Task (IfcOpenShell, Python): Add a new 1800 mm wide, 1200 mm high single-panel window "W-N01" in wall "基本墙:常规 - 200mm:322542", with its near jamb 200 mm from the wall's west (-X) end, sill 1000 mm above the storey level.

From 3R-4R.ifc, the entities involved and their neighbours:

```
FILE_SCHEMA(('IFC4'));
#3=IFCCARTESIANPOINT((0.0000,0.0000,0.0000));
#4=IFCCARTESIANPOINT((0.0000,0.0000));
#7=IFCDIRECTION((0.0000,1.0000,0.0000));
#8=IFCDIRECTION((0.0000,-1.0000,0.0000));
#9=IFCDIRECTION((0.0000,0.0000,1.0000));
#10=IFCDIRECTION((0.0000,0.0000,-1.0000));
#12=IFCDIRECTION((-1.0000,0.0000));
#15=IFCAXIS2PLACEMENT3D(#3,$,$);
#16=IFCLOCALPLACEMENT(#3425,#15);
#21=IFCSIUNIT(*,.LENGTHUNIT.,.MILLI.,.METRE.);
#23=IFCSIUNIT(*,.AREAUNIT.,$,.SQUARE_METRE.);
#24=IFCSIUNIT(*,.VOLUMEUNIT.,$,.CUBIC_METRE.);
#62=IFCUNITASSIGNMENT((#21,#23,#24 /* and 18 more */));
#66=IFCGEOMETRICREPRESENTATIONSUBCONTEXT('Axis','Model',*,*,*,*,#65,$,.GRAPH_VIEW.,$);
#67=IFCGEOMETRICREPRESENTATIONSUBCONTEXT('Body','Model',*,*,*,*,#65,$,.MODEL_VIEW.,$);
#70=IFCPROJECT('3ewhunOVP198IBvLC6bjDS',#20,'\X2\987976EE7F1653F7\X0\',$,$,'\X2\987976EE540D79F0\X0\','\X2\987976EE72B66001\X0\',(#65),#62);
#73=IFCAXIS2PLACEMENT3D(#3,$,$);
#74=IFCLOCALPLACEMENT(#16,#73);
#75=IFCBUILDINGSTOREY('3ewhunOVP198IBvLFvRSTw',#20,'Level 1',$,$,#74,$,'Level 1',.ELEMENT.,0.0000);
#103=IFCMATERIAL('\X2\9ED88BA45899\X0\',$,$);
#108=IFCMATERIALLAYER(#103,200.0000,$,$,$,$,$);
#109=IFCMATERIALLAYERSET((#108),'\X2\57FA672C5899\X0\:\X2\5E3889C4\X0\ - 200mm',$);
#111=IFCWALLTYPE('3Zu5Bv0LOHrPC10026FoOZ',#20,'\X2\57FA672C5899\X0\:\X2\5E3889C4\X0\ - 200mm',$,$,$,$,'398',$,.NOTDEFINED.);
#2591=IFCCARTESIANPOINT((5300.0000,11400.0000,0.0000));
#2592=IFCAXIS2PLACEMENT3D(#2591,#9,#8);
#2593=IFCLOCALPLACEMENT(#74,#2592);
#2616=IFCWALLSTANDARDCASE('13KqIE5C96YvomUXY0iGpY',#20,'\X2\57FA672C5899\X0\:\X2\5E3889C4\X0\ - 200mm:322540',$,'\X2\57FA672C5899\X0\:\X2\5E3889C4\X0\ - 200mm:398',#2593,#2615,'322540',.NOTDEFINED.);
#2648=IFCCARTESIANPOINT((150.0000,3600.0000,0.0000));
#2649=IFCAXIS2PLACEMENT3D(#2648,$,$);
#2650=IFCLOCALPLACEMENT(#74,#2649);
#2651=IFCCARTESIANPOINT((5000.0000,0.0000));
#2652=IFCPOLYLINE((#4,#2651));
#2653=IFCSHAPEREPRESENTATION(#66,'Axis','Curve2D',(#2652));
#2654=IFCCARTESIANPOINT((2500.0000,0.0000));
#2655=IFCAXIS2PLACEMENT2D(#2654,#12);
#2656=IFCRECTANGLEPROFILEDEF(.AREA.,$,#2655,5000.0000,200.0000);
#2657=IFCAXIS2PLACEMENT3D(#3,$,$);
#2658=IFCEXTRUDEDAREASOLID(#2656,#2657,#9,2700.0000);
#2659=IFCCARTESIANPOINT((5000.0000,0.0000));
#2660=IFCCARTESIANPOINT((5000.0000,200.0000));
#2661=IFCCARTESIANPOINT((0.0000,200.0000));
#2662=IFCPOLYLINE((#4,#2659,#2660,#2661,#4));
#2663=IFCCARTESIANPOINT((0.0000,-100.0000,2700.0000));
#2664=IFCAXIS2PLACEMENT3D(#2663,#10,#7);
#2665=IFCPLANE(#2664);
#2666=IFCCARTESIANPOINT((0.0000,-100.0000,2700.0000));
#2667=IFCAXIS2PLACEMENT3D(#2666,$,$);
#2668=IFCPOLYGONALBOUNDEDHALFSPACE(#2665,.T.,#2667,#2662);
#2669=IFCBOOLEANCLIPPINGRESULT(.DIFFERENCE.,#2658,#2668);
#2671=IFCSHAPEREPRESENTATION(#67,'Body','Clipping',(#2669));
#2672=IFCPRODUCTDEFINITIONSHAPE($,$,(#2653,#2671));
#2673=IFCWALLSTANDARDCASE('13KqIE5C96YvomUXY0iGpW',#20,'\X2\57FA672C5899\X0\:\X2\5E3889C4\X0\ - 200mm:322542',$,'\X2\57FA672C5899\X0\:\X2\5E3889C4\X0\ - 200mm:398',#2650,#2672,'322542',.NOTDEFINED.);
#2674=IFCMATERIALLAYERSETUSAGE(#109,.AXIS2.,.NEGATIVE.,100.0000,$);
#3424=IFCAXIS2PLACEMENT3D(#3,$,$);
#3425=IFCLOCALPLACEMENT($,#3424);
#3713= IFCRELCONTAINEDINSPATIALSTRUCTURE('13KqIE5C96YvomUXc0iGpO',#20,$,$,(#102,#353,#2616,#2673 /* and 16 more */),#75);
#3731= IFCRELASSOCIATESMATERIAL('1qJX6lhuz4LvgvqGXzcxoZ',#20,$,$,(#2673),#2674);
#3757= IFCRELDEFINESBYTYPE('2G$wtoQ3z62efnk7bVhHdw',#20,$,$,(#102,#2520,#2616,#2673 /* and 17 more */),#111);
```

```python
import numpy as np
import ifcopenshell
import ifcopenshell.api.feature
import ifcopenshell.api.geometry
import ifcopenshell.api.root
import ifcopenshell.api.spatial
import ifcopenshell.geom
import ifcopenshell.util.element
import ifcopenshell.util.placement
import ifcopenshell.util.representation
import ifcopenshell.util.shape
import ifcopenshell.util.unit

model = ifcopenshell.open("3R-4R.ifc")
unit_scale = ifcopenshell.util.unit.calculate_unit_scale(model)
settings = ifcopenshell.geom.settings()


def volume(element):
    """Net volume in cubic metres, openings subtracted."""
    shape = ifcopenshell.geom.create_shape(settings, element)
    return ifcopenshell.util.shape.get_volume(shape.geometry)


wall = model.by_guid("13KqIE5C96YvomUXY0iGpW")
storey = ifcopenshell.util.element.get_container(wall, ifc_class="IfcBuildingStorey")
context = ifcopenshell.util.representation.get_context(model, "Model", "Body", "MODEL_VIEW")
before = volume(wall)

width, height, from_end, sill = 1.8, 1.2, 0.2, 1  # metres

# The wall runs along its own X axis, and the end named is its -X end.
wall_shape = ifcopenshell.geom.create_shape(settings, wall)
x, y, z = ifcopenshell.util.shape.get_vertices(wall_shape.geometry).T
start = x.min() + from_end
face, thickness = float(y.min()), float(y.max() - y.min())
wall_matrix = ifcopenshell.util.placement.get_local_placement(wall.ObjectPlacement)
level = ifcopenshell.util.placement.get_local_placement(storey.ObjectPlacement)[2, 3]


def in_wall(x, y):
    """Placement at x, y metres in the wall's axes, at sill height."""
    matrix = wall_matrix.copy()
    matrix[:, 3] = wall_matrix @ np.array([x / unit_scale, y / unit_scale, 0.0, 1.0])
    matrix[2, 3] = level + sill / unit_scale
    return matrix


# Opening: a box that overshoots both wall faces by 50 mm.
opening = ifcopenshell.api.root.create_entity(model, ifc_class="IfcOpeningElement", predefined_type="OPENING")
box = ifcopenshell.api.geometry.add_wall_representation(
    model, context=context, length=width, height=height, thickness=thickness + 0.1
)
ifcopenshell.api.geometry.assign_representation(model, product=opening, representation=box)
ifcopenshell.api.geometry.edit_object_placement(model, product=opening, matrix=in_wall(start, face - 0.05), is_si=False)
ifcopenshell.api.feature.add_feature(model, feature=opening, element=wall)

window = ifcopenshell.api.root.create_entity(model, ifc_class="IfcWindow", name="W-N01", predefined_type="WINDOW")
window.OverallWidth, window.OverallHeight = width / unit_scale, height / unit_scale
window.PartitioningType = "SINGLE_PANEL"
body = ifcopenshell.api.geometry.add_window_representation(
    model,
    context=context,
    overall_width=window.OverallWidth,
    overall_height=window.OverallHeight,
    partition_type="SINGLE_PANEL",
)
ifcopenshell.api.geometry.assign_representation(model, product=window, representation=body)
ifcopenshell.api.spatial.assign_container(model, products=[window], relating_structure=storey)
ifcopenshell.api.feature.add_filling(model, opening=opening, element=window)

# Centre the window in the wall's thickness.
ifcopenshell.api.geometry.edit_object_placement(model, product=window, matrix=in_wall(start, face), is_si=False)
window_shape = ifcopenshell.geom.create_shape(settings, window)
depth = ifcopenshell.util.shape.get_vertices(window_shape.geometry)[:, 1]
offset = face + thickness / 2 - (depth.min() + depth.max()) / 2
ifcopenshell.api.geometry.edit_object_placement(model, product=window, matrix=in_wall(start, offset), is_si=False)

after = volume(wall)

print(f"wall volume {before:.3f} -> {after:.3f} m3")

model.write("3R-4R_edited.ifc")
```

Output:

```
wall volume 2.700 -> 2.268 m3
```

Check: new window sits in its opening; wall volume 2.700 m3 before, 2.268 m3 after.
